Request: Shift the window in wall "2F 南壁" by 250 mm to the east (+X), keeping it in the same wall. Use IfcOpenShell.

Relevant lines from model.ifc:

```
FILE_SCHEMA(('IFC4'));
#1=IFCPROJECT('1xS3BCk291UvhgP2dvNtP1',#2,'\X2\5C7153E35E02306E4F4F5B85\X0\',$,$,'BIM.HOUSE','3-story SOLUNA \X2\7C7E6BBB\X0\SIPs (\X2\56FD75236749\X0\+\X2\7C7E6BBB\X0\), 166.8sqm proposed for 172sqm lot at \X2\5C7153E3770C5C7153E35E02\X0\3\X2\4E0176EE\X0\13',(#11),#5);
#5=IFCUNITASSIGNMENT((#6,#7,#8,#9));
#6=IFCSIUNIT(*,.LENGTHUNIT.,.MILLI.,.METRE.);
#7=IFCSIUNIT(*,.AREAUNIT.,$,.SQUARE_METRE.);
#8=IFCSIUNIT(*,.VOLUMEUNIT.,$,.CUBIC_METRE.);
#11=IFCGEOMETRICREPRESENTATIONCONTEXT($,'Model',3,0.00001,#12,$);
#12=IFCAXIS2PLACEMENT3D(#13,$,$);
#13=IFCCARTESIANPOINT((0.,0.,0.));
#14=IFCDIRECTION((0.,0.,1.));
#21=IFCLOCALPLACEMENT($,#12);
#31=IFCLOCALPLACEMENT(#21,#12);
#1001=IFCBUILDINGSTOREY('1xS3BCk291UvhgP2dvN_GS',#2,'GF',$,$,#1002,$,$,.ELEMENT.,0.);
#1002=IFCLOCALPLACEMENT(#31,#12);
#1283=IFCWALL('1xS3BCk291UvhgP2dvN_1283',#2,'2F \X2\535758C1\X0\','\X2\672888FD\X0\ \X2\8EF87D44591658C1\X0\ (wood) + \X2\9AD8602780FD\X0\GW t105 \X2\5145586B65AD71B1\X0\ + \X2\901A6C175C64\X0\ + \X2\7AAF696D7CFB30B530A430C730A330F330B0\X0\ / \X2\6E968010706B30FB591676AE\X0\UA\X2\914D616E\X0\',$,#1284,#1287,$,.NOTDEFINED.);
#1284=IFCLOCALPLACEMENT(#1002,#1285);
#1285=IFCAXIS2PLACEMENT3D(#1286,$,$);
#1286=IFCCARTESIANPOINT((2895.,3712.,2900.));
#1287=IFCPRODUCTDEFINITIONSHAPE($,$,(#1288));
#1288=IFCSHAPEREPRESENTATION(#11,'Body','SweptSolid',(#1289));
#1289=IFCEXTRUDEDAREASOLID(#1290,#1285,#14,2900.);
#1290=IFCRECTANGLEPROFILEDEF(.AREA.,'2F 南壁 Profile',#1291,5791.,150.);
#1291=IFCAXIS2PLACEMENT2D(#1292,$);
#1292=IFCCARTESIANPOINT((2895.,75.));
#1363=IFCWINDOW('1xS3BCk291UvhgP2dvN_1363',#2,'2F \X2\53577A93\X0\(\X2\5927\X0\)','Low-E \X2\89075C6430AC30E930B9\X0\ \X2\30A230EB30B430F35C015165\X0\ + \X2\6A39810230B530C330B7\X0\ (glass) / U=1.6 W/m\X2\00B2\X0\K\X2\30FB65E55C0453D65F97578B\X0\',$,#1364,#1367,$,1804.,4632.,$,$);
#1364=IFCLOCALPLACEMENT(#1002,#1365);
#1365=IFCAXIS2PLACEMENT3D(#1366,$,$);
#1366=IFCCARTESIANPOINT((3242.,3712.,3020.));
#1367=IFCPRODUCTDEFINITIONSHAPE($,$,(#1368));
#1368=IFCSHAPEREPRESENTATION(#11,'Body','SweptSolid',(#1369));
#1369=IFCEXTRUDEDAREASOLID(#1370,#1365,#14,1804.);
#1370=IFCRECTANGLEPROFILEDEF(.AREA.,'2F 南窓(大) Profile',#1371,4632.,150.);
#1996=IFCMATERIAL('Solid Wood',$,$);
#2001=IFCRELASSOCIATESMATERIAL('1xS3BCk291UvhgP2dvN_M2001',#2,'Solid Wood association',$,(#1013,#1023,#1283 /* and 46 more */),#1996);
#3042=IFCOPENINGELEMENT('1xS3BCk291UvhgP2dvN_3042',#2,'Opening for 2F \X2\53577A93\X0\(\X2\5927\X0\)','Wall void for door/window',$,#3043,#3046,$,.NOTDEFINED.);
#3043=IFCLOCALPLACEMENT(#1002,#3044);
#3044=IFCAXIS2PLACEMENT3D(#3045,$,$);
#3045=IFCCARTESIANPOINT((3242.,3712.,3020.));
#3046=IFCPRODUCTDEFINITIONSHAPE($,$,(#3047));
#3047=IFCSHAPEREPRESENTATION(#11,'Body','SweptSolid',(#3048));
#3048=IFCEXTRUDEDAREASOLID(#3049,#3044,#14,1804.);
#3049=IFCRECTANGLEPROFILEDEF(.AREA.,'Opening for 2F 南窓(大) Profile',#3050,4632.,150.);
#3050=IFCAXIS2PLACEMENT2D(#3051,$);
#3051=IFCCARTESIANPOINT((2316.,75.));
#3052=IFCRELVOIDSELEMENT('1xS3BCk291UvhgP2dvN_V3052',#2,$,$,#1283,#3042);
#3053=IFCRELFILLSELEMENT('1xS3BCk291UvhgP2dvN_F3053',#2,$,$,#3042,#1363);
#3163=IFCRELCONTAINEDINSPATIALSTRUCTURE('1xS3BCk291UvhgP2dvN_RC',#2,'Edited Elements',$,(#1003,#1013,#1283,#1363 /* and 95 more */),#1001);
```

```python
import ifcopenshell
import ifcopenshell.api.geometry
import ifcopenshell.util.placement
import ifcopenshell.util.unit

model = ifcopenshell.open("model.ifc")
unit_scale = ifcopenshell.util.unit.calculate_unit_scale(model)

window = model.by_guid("1xS3BCk291UvhgP2dvN_1363")
opening = window.FillsVoids[0].RelatingOpeningElement
wall = opening.VoidsElements[0].RelatingBuildingElement

wall_matrix = ifcopenshell.util.placement.get_local_placement(wall.ObjectPlacement)
shift = wall_matrix[:3, 0] * 0.25 / unit_scale
before = ifcopenshell.util.placement.get_local_placement(window.ObjectPlacement)[:3, 3].copy()

# The window is not placed relative to its opening, so move both.
for product in (opening, window):
    matrix = ifcopenshell.util.placement.get_local_placement(product.ObjectPlacement)
    matrix[:3, 3] += shift
    ifcopenshell.api.geometry.edit_object_placement(model, product=product, matrix=matrix, is_si=False)

after = ifcopenshell.util.placement.get_local_placement(window.ObjectPlacement)[:3, 3]
print("window moved by", (after - before).round(3) + 0.0)

model.write("model_edited.ifc")
```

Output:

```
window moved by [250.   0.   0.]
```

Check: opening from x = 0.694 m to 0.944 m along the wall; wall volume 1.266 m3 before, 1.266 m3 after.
